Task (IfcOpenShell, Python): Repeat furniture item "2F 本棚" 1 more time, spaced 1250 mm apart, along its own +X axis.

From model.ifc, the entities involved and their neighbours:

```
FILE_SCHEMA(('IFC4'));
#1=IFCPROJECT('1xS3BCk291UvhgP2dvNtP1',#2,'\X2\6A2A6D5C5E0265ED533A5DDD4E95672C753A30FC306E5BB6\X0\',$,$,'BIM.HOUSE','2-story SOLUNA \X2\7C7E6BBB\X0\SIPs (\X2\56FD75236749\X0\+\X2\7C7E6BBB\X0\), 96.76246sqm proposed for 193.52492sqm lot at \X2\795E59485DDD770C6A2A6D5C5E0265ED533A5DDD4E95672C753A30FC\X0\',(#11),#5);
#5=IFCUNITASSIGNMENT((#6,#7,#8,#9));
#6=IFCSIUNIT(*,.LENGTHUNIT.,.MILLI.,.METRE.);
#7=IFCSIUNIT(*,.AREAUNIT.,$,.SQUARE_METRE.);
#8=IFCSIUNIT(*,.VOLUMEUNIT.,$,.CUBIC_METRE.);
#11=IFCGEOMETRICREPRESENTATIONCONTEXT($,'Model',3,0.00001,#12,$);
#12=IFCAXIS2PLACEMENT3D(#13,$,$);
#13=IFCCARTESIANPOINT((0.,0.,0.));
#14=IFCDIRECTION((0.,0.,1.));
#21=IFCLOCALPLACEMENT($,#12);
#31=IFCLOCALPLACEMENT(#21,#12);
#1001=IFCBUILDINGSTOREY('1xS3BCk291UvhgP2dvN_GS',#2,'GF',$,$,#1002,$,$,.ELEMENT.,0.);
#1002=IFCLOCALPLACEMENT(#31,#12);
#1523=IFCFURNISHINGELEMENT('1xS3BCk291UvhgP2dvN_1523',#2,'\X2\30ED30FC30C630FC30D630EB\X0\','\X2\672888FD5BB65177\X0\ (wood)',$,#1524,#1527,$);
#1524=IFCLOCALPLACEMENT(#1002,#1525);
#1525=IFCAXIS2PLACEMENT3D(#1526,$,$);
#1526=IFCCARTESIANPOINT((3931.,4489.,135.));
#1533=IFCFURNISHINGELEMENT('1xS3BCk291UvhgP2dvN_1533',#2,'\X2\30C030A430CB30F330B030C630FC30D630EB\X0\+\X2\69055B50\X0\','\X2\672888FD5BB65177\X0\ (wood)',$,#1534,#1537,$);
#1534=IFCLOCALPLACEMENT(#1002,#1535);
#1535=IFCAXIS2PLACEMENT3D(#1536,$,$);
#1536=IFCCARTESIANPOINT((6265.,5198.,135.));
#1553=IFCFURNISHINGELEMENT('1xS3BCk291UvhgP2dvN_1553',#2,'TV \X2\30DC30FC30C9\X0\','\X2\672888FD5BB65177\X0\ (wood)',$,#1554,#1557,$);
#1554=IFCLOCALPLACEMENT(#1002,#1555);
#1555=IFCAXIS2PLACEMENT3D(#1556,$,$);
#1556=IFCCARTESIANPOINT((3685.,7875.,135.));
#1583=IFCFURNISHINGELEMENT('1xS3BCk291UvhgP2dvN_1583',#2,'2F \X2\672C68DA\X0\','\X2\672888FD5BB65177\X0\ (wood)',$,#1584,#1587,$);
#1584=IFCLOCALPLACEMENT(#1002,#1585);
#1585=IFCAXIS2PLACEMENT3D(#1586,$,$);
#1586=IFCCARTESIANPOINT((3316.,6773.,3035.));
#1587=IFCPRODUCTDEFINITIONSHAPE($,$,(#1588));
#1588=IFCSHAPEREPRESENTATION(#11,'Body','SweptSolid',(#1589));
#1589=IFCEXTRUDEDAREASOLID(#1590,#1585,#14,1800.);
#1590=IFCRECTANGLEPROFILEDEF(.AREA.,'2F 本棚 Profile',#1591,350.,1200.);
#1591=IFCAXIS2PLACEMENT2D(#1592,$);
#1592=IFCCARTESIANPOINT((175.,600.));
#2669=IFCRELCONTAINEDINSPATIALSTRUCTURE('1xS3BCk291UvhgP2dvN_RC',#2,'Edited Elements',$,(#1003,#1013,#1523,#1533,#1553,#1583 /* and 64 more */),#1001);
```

```python
import ifcopenshell
import ifcopenshell.api.geometry
import ifcopenshell.api.root
import ifcopenshell.util.element
import ifcopenshell.util.placement

model = ifcopenshell.open("model.ifc")


def reuse_history(source, copy):
    """copy_class also copies each property set's owner history, people and application; keep the originals."""
    for rel in copy.IsDefinedBy:
        if rel.is_a("IfcRelDefinesByProperties") and (history := rel.RelatingPropertyDefinition.OwnerHistory):
            rel.RelatingPropertyDefinition.OwnerHistory = source.OwnerHistory
            ifcopenshell.util.element.remove_deep2(model, history)


source = model.by_guid("1xS3BCk291UvhgP2dvN_1583")
base = ifcopenshell.util.placement.get_local_placement(source.ObjectPlacement)
step = base[:3, 0] * 1250.0

for i in range(1, 2):
    copy = ifcopenshell.api.root.copy_class(model, product=source)
    copy.Representation = ifcopenshell.util.element.copy_deep(
        model, source.Representation, exclude=["IfcGeometricRepresentationContext", "IfcRepresentationMap"]
    )
    reuse_history(source, copy)
    matrix = base.copy()
    matrix[:3, 3] += i * step
    print("added at", matrix[:3, 3].round(3) + 0.0)
    ifcopenshell.api.geometry.edit_object_placement(model, product=copy, matrix=matrix, is_si=False)

model.write("model_v2.ifc")
```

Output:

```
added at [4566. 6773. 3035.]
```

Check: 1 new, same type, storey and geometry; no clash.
